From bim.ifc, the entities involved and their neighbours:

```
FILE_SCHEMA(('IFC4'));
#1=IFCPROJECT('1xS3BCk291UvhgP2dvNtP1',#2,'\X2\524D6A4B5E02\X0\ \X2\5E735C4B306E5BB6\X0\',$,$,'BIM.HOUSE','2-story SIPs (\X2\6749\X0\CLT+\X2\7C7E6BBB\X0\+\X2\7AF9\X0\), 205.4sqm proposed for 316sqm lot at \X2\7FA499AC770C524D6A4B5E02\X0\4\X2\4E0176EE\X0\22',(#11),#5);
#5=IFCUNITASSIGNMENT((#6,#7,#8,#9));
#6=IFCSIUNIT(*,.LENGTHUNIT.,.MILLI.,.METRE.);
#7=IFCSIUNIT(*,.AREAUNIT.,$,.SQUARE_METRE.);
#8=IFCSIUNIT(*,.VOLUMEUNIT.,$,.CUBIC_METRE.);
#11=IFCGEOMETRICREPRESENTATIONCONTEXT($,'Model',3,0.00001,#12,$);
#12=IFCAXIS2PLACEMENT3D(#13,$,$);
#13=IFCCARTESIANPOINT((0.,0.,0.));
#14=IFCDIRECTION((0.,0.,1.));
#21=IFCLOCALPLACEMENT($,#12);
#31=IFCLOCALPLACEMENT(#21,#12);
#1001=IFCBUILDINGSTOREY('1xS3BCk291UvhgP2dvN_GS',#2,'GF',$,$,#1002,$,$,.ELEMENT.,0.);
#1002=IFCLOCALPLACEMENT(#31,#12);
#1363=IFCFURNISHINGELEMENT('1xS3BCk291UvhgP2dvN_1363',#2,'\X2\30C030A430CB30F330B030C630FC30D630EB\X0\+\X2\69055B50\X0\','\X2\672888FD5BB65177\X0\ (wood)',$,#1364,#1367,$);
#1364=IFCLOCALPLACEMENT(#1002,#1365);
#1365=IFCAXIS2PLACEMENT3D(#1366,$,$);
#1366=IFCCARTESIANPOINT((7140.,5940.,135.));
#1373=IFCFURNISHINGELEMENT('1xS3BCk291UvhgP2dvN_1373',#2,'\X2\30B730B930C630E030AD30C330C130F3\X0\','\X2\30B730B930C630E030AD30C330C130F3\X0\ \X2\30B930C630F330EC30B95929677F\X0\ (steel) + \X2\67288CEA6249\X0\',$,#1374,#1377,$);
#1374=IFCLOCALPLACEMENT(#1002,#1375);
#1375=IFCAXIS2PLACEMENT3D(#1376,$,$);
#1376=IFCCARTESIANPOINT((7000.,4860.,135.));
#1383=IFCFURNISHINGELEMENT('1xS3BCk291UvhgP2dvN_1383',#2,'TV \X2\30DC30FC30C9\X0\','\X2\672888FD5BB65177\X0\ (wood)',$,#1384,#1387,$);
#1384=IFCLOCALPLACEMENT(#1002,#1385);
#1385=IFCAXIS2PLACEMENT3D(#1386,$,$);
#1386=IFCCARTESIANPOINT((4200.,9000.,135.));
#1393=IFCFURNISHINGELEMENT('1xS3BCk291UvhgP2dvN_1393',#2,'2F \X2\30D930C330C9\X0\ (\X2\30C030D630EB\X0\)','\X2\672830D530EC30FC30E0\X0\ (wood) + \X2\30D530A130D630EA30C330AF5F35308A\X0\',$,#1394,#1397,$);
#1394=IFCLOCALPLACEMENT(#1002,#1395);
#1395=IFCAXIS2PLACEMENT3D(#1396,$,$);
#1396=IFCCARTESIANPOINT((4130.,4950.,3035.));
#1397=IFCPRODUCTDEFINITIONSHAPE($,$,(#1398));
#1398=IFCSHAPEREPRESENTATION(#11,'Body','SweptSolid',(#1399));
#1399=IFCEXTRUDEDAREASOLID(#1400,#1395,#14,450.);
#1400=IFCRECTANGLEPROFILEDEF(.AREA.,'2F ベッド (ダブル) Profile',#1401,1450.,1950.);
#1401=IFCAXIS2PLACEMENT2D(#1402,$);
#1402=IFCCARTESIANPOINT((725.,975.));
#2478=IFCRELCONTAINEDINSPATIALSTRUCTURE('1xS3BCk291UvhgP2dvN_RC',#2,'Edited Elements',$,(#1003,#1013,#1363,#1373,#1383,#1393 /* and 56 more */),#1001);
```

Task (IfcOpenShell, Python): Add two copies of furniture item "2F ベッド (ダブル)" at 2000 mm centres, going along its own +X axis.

```python
import ifcopenshell
import ifcopenshell.api.geometry
import ifcopenshell.api.root
import ifcopenshell.util.element
import ifcopenshell.util.placement

model = ifcopenshell.open("bim.ifc")


def reuse_history(source, copy):
    """copy_class also copies each property set's owner history, people and application; keep the originals."""
    for rel in copy.IsDefinedBy:
        if rel.is_a("IfcRelDefinesByProperties") and (history := rel.RelatingPropertyDefinition.OwnerHistory):
            rel.RelatingPropertyDefinition.OwnerHistory = source.OwnerHistory
            ifcopenshell.util.element.remove_deep2(model, history)


source = model.by_guid("1xS3BCk291UvhgP2dvN_1393")
base = ifcopenshell.util.placement.get_local_placement(source.ObjectPlacement)
step = base[:3, 0] * 2000.0

for i in range(1, 3):
    copy = ifcopenshell.api.root.copy_class(model, product=source)
    copy.Representation = ifcopenshell.util.element.copy_deep(
        model, source.Representation, exclude=["IfcGeometricRepresentationContext", "IfcRepresentationMap"]
    )
    reuse_history(source, copy)
    matrix = base.copy()
    matrix[:3, 3] += i * step
    print("added at", matrix[:3, 3].round(3) + 0.0)
    ifcopenshell.api.geometry.edit_object_placement(model, product=copy, matrix=matrix, is_si=False)

model.write("bim_edited.ifc")
```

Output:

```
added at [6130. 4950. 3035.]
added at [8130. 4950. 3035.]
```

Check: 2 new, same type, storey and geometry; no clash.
